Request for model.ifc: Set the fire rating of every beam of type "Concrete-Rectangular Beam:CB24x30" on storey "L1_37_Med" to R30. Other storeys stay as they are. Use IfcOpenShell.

First a look at what the model holds.

```python
import ifcopenshell
import ifcopenshell.util.element

model = ifcopenshell.open("model.ifc")
print(model.schema)
storey = next(s for s in model.by_type("IfcBuildingStorey") if s.Name == "L1_37_Med")
beams = [e for e in ifcopenshell.util.element.get_decomposition(storey) if e.is_a("IfcBeam")]
seen = {}
for e in beams:
    element_type = ifcopenshell.util.element.get_type(e)
    key = (element_type.Name if element_type != e and element_type else None, ifcopenshell.util.element.get_pset(e, "Pset_BeamCommon", "FireRating"))
    seen[key] = seen.get(key, 0) + 1
for (name, value), count in sorted(seen.items(), key=str):
    print(count, "x", name, "|", value)
```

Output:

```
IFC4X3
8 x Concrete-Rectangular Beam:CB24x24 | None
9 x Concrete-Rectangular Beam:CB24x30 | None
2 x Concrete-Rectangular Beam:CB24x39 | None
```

```python
import ifcopenshell
import ifcopenshell.api.pset
import ifcopenshell.util.element

model = ifcopenshell.open("model.ifc")

storey = next(s for s in model.by_type("IfcBuildingStorey") if s.Name == "L1_37_Med")
beams = [e for e in ifcopenshell.util.element.get_decomposition(storey) if e.is_a("IfcBeam")]

count = 0
for e in beams:
    element_type = ifcopenshell.util.element.get_type(e)
    if element_type in (None, e) or element_type.Name != "Concrete-Rectangular Beam:CB24x30":
        continue
    # add_pset returns the element's existing set when there is one.
    pset = ifcopenshell.api.pset.add_pset(model, product=e, name="Pset_BeamCommon")
    ifcopenshell.api.pset.edit_pset(model, pset=pset, properties={"FireRating": "R30"})
    count += 1

print(count, "beams updated")

model.write("model_updated.ifc")
```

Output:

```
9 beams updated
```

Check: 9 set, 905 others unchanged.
